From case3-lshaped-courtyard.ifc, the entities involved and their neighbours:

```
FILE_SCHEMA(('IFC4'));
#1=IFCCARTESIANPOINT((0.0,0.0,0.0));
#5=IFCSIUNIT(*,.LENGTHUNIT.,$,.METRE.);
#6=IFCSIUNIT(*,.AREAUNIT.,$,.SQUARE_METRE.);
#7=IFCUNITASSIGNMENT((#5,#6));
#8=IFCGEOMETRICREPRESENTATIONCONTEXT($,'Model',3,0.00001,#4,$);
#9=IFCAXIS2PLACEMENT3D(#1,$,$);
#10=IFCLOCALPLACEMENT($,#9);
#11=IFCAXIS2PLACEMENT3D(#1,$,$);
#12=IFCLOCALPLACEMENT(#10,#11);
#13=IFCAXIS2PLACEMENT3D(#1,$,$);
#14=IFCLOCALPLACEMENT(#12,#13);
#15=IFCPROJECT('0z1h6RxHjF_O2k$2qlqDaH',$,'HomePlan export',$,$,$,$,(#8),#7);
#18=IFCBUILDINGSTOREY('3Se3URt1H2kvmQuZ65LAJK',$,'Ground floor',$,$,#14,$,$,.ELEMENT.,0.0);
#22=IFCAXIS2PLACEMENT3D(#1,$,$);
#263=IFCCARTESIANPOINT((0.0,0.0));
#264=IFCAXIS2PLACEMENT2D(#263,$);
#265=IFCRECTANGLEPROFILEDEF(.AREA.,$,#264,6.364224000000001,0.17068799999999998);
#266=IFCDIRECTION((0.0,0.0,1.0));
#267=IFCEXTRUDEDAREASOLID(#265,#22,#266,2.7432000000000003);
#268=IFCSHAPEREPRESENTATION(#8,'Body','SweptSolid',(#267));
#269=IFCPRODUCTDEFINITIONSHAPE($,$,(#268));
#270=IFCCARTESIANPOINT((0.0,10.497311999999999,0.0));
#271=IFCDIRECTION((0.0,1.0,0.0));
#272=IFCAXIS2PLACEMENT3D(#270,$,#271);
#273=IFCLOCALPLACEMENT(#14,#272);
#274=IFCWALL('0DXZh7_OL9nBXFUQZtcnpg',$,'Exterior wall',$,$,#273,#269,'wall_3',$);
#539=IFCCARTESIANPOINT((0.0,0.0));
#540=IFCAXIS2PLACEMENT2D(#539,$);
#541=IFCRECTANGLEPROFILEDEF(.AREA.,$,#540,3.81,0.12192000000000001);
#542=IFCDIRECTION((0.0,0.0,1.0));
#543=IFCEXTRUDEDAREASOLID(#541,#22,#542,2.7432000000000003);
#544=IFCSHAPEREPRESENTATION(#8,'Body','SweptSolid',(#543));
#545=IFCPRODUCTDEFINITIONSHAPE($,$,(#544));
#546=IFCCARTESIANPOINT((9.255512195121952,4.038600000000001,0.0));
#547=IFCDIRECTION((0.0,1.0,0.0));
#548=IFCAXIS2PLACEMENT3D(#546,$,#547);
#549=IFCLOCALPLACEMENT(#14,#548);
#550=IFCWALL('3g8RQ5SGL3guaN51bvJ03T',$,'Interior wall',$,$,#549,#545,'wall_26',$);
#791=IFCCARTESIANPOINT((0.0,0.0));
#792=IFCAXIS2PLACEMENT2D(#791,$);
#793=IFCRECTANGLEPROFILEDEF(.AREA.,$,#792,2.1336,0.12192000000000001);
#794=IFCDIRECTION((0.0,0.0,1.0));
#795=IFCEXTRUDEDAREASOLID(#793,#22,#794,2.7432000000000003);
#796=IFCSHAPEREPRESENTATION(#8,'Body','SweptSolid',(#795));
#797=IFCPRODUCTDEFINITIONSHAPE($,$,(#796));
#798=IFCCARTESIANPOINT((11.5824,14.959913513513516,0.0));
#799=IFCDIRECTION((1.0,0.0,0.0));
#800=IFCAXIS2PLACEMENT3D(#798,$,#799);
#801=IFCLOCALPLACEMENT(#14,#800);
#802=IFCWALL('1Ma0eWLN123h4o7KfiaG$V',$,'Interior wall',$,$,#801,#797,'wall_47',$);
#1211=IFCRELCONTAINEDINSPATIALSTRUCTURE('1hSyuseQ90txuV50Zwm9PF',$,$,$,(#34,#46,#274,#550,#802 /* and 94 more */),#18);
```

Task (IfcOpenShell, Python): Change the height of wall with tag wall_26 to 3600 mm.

```python
import ifcopenshell
import ifcopenshell.geom
import ifcopenshell.util.shape
import ifcopenshell.util.unit

model = ifcopenshell.open("case3-lshaped-courtyard.ifc")
unit_scale = ifcopenshell.util.unit.calculate_unit_scale(model)
settings = ifcopenshell.geom.settings()


def volume(element):
    """Net volume in cubic metres, openings subtracted."""
    shape = ifcopenshell.geom.create_shape(settings, element)
    return ifcopenshell.util.shape.get_volume(shape.geometry)


wall = model.by_id(550)
before = volume(wall)

body = next(r for r in wall.Representation.Representations if r.RepresentationIdentifier == "Body")
solid = body.Items[0]
old_height = solid.Depth
solid.Depth = 3.6 / unit_scale
after = volume(wall)

print(f"height {old_height:g} -> {solid.Depth:g}, volume {before:.3f} -> {after:.3f} m3")

model.write("case3-lshaped-courtyard_updated.ifc")
```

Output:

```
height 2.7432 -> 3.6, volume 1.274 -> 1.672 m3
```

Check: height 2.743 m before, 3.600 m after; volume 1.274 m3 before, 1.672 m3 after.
